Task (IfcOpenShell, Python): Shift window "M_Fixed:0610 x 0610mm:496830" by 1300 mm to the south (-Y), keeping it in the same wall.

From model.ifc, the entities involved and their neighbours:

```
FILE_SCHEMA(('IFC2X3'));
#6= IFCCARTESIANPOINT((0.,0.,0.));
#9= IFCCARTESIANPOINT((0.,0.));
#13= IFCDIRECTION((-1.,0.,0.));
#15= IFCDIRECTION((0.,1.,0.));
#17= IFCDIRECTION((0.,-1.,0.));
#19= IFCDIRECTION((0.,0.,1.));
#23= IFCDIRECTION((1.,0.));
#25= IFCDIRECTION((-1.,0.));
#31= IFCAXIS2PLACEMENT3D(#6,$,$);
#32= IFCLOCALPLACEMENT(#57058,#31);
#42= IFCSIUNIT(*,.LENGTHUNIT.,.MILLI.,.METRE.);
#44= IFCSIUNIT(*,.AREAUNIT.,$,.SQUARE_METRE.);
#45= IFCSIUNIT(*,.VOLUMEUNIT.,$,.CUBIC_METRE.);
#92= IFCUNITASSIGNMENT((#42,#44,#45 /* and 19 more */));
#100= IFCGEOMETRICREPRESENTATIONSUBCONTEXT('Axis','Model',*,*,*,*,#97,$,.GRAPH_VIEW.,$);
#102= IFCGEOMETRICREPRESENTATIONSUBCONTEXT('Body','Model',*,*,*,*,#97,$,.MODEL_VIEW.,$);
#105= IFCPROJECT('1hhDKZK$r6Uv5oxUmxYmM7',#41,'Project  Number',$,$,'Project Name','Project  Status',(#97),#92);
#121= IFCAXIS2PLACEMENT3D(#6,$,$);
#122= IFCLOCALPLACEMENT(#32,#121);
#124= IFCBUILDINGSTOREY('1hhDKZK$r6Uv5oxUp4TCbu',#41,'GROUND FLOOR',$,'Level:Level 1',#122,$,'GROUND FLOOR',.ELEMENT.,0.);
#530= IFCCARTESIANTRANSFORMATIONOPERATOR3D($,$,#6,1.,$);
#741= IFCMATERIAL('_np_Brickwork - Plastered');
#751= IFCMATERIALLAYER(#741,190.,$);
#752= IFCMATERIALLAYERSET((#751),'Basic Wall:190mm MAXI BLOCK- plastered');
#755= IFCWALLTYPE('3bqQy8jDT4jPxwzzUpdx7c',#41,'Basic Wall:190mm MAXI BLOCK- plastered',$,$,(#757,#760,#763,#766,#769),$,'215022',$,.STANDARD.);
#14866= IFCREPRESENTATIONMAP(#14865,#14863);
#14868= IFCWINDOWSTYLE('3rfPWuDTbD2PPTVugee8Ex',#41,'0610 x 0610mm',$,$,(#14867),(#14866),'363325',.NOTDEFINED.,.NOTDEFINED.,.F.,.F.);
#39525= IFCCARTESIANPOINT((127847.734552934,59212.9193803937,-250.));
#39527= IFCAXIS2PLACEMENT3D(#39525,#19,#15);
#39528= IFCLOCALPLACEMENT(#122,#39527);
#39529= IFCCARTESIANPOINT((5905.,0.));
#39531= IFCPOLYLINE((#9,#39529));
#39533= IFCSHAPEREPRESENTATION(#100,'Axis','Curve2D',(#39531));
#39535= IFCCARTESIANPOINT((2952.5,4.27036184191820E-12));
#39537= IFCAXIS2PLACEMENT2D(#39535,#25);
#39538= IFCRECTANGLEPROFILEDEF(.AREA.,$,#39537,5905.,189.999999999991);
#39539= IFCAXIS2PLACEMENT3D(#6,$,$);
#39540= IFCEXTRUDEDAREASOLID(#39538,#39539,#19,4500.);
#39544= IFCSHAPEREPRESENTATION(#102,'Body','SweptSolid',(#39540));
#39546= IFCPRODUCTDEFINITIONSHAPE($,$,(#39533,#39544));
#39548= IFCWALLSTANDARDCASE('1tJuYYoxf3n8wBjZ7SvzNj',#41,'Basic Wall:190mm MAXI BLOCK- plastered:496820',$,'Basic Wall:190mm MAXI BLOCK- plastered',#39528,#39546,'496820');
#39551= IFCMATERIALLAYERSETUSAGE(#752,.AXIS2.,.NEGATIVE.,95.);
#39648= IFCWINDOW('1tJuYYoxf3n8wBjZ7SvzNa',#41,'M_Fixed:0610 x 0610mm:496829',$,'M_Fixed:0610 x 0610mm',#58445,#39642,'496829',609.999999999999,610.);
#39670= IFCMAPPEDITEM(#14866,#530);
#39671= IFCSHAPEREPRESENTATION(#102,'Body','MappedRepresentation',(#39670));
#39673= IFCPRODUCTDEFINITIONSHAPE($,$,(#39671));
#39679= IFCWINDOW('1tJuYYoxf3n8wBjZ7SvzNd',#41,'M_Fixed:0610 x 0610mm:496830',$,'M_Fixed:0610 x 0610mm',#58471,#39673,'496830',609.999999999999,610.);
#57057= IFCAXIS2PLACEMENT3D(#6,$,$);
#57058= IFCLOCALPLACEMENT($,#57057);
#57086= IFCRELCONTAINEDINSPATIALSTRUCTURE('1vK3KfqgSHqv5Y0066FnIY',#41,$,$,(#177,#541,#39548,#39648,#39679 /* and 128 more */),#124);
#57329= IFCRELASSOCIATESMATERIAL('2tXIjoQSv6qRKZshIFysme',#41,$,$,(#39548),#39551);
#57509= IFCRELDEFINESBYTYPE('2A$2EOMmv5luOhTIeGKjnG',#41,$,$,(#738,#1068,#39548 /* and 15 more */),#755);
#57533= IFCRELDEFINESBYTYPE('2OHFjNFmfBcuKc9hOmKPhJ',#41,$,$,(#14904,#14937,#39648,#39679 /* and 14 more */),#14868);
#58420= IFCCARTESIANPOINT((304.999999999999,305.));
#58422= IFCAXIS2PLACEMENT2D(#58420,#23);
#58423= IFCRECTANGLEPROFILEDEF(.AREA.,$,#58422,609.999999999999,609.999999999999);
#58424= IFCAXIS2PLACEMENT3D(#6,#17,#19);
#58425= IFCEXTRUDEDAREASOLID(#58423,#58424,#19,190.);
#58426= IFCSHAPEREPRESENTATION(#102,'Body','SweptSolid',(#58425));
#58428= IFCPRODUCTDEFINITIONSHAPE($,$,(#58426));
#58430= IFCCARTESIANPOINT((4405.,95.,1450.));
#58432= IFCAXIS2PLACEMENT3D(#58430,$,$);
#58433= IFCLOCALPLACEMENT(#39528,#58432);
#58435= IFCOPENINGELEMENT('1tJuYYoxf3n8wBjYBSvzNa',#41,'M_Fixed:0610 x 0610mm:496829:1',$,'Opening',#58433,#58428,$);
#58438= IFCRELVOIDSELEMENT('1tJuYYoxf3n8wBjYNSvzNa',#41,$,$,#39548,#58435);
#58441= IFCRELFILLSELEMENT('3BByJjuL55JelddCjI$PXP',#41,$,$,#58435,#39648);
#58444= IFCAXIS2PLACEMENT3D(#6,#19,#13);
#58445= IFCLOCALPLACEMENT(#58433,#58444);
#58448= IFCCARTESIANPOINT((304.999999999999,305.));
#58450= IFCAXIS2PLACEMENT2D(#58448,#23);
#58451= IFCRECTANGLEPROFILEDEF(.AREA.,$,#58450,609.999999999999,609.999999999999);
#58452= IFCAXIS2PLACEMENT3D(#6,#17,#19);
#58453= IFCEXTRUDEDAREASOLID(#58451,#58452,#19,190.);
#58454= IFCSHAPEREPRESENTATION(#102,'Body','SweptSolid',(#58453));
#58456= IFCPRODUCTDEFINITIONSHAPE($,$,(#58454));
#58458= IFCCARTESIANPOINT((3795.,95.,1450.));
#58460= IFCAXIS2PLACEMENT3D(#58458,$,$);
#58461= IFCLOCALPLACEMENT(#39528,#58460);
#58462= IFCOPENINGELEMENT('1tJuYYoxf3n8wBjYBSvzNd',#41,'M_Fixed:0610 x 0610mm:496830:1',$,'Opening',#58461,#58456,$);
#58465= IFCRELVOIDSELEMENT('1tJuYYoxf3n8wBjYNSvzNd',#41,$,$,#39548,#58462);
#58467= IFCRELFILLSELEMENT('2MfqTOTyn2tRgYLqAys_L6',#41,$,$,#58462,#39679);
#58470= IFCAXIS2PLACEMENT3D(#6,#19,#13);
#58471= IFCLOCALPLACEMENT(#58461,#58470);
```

```python
import ifcopenshell
import ifcopenshell.api.geometry
import ifcopenshell.util.placement

model = ifcopenshell.open("model.ifc")

window = model.by_guid("1tJuYYoxf3n8wBjZ7SvzNd")
opening = window.FillsVoids[0].RelatingOpeningElement
wall = opening.VoidsElements[0].RelatingBuildingElement

wall_matrix = ifcopenshell.util.placement.get_local_placement(wall.ObjectPlacement)
shift = wall_matrix[:3, 0] * -1300.0
before = ifcopenshell.util.placement.get_local_placement(window.ObjectPlacement)[:3, 3].copy()

# The window is placed relative to its opening, so it follows when the opening moves.
matrix = ifcopenshell.util.placement.get_local_placement(opening.ObjectPlacement)
matrix[:3, 3] += shift
ifcopenshell.api.geometry.edit_object_placement(
    model, product=opening, matrix=matrix, is_si=False, should_transform_children=True
)

after = ifcopenshell.util.placement.get_local_placement(window.ObjectPlacement)[:3, 3]
print("window moved by", (after - before).round(3) + 0.0)

model.write("model-out.ifc")
```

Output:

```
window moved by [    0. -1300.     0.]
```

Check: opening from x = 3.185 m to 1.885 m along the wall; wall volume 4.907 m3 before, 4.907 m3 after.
